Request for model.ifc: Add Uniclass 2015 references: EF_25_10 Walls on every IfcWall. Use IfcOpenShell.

First a look at what the model holds.

```python
import ifcopenshell

model = ifcopenshell.open("model.ifc")
print(model.schema)
print("classifications:", [c.Name for c in model.by_type("IfcClassification")])
for ifc_class in ("IfcDoor", "IfcRoof", "IfcStair", "IfcWall", "IfcWindow"):
    print(ifc_class, len(model.by_type(ifc_class)))
```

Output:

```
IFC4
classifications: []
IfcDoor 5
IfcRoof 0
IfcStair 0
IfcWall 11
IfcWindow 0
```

```python
import ifcopenshell
import ifcopenshell.api.classification

model = ifcopenshell.open("model.ifc")

system = ifcopenshell.api.classification.add_classification(model, classification="Uniclass 2015")

codes = {
    "IfcWall": ("EF_25_10", "Walls"),
}
for ifc_class, (code, name) in codes.items():
    products = model.by_type(ifc_class)
    ifcopenshell.api.classification.add_reference(
        model, products=products, classification=system, identification=code, name=name
    )
    print(code, len(products))

model.write("model_rev.ifc")
```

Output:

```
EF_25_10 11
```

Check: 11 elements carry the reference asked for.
